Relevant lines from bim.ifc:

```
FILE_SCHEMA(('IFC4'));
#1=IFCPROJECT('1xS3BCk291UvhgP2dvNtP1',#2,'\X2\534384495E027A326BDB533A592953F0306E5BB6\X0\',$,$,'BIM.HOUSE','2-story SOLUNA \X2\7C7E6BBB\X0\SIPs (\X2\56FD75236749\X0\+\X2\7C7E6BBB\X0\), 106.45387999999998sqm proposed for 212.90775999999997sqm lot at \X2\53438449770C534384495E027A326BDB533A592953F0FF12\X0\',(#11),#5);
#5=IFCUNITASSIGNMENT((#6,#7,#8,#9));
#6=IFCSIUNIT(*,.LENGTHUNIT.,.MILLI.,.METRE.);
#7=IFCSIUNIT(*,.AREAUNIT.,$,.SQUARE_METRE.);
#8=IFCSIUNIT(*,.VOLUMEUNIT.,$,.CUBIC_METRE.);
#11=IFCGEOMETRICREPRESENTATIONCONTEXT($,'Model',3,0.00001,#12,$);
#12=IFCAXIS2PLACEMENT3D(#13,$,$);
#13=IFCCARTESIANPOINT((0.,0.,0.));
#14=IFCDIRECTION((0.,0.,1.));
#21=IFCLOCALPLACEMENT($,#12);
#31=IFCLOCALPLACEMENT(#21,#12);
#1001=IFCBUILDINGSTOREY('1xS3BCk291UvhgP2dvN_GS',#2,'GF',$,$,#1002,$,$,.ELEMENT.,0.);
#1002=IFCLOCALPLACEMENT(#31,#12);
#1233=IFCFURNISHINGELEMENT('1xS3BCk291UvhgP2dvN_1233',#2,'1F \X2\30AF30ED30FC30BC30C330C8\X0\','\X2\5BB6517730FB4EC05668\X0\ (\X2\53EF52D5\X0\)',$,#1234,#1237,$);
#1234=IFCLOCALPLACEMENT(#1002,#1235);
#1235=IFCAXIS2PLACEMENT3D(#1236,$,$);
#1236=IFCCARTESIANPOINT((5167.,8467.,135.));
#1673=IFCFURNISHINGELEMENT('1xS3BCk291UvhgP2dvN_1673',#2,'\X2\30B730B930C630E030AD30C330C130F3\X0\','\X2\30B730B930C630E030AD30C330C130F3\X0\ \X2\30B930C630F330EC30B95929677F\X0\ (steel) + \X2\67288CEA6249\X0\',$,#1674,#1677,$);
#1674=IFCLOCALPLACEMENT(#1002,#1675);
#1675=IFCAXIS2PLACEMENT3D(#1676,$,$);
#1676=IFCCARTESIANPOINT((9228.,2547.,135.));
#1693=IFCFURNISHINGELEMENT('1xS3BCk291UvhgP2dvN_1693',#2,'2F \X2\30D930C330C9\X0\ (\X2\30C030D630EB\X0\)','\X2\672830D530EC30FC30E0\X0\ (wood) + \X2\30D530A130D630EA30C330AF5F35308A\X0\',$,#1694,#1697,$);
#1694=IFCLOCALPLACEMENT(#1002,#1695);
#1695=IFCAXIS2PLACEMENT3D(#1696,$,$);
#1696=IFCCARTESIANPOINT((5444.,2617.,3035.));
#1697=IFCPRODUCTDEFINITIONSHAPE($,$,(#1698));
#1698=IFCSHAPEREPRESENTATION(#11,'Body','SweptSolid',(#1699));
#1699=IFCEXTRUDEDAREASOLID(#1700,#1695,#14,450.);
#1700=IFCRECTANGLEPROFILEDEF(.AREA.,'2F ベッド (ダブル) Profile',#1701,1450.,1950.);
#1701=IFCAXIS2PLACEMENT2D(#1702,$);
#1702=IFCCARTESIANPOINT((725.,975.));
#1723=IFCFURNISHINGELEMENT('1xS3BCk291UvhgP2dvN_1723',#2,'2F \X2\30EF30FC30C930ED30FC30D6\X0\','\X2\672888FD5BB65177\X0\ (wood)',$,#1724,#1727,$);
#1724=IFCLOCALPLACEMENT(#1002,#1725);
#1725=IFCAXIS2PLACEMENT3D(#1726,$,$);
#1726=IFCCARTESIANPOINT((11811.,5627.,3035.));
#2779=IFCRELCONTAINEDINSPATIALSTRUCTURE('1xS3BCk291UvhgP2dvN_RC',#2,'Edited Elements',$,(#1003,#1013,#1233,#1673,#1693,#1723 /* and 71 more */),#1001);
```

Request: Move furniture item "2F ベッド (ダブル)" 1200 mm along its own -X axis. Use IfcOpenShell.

```python
import ifcopenshell
import ifcopenshell.api.geometry
import ifcopenshell.util.placement
import ifcopenshell.util.unit

model = ifcopenshell.open("bim.ifc")
unit_scale = ifcopenshell.util.unit.calculate_unit_scale(model)

item = model.by_id(1693)
matrix = ifcopenshell.util.placement.get_local_placement(item.ObjectPlacement)
matrix[:3, 3] -= matrix[:3, 0] * 1.2 / unit_scale
ifcopenshell.api.geometry.edit_object_placement(model, product=item, matrix=matrix, is_si=False)

print(ifcopenshell.util.placement.get_local_placement(item.ObjectPlacement).round(3) + 0.0)

model.write("bim-out.ifc")
```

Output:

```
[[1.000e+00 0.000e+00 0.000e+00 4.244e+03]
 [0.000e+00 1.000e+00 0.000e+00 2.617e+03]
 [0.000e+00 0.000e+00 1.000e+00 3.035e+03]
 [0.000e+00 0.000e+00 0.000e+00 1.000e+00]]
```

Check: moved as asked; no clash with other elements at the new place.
